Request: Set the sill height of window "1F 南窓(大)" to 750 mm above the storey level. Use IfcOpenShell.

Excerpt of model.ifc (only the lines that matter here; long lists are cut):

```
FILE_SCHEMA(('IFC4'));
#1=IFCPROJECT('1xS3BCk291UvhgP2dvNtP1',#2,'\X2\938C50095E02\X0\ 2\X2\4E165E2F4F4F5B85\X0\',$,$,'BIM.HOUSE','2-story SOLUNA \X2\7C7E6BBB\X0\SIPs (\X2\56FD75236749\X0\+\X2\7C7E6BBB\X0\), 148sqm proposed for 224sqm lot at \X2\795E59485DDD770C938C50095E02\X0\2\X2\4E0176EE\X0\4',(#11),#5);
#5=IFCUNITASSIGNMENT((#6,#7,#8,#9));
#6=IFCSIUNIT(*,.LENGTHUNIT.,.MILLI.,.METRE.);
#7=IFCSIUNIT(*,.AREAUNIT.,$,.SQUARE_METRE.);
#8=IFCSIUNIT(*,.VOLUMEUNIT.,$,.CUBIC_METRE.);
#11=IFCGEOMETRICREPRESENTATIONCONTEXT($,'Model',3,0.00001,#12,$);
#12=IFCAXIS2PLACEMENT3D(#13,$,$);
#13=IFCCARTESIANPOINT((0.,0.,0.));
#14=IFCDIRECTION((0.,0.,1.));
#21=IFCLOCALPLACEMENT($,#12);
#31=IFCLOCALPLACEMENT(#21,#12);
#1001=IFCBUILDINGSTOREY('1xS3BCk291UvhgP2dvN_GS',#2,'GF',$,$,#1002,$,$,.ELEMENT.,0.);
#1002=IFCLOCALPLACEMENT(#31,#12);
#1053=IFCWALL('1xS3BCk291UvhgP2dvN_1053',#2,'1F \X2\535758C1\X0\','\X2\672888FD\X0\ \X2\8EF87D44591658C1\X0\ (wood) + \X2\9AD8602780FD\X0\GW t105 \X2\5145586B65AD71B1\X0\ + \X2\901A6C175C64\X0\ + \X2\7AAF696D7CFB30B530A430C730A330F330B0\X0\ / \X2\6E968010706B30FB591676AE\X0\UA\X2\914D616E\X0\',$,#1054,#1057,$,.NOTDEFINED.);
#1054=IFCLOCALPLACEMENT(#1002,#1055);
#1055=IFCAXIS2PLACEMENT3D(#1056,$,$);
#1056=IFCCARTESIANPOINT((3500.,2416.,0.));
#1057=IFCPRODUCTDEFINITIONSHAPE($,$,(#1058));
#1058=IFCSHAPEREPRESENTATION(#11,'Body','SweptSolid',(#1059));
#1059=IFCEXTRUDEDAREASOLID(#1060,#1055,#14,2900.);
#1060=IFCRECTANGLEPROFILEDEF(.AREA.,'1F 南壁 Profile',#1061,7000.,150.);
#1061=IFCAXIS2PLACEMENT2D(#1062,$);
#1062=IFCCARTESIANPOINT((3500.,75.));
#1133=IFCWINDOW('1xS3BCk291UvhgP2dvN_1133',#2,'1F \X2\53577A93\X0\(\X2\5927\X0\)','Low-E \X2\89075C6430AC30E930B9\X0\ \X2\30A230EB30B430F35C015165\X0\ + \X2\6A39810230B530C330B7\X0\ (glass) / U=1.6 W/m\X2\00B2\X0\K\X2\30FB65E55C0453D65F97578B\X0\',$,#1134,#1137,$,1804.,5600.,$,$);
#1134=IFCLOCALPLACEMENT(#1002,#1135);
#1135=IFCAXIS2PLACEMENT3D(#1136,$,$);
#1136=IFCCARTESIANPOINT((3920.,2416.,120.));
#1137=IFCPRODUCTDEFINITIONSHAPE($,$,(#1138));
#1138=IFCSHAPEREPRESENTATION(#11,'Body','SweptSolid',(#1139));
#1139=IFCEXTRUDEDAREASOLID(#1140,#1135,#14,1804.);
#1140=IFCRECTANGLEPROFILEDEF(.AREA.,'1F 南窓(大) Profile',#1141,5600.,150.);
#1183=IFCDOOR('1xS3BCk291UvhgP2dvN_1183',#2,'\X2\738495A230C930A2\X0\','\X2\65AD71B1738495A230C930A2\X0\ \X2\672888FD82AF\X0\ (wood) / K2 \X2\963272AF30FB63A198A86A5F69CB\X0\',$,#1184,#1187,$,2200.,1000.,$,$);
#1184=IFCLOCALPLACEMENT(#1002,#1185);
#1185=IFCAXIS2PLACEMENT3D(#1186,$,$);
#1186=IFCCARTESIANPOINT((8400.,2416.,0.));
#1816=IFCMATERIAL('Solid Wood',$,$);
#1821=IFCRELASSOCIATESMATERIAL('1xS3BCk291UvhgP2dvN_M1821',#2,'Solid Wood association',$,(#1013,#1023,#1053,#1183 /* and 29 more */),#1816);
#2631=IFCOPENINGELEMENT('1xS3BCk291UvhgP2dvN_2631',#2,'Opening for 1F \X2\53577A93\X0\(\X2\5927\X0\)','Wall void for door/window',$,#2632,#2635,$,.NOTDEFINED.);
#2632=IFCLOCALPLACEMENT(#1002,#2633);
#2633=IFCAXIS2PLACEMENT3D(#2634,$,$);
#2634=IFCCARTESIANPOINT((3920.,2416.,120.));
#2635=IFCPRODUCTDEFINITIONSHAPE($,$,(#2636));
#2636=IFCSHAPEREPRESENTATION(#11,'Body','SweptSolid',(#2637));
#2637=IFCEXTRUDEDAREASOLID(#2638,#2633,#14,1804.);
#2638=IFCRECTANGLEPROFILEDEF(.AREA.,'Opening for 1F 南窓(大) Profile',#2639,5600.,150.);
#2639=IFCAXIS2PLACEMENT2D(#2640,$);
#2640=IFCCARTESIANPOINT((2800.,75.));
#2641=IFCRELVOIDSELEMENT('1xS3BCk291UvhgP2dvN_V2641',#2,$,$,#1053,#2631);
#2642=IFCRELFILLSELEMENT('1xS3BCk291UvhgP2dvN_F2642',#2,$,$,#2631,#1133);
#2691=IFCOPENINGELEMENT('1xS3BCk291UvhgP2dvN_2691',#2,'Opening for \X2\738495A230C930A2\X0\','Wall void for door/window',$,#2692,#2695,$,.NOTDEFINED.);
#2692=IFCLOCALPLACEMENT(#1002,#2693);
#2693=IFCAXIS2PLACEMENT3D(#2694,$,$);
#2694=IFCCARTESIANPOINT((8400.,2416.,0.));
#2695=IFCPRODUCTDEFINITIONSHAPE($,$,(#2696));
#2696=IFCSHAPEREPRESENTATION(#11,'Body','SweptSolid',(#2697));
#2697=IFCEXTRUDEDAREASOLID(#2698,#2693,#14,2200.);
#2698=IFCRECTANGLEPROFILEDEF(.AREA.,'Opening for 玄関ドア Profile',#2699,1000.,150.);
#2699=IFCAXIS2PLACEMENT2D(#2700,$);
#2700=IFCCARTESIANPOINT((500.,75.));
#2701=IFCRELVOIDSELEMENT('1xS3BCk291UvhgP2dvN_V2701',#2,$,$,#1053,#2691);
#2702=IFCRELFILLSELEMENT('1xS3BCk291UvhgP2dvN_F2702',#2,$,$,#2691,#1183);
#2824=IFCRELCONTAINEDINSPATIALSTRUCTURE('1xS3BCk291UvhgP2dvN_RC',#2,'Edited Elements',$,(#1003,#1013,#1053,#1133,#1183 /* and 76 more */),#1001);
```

```python
import numpy as np
import ifcopenshell
import ifcopenshell.api.geometry
import ifcopenshell.geom
import ifcopenshell.util.element
import ifcopenshell.util.placement
import ifcopenshell.util.shape
import ifcopenshell.util.unit

model = ifcopenshell.open("model.ifc")
unit_scale = ifcopenshell.util.unit.calculate_unit_scale(model)

window = model.by_guid("1xS3BCk291UvhgP2dvN_1133")
opening = window.FillsVoids[0].RelatingOpeningElement
storey = ifcopenshell.util.element.get_container(window, ifc_class="IfcBuildingStorey")
level = ifcopenshell.util.placement.get_local_placement(storey.ObjectPlacement)[2, 3]

# The opening's origin need not be at the sill, so measure its lowest point.
shape = ifcopenshell.geom.create_shape(ifcopenshell.geom.settings(), opening)
bottom = ifcopenshell.util.shape.get_shape_bottom_elevation(shape, shape.geometry) / unit_scale
dz = level + 0.75 / unit_scale - bottom

shift = np.array([0.0, 0.0, dz])
# The window is not placed relative to its opening, so move both.
for product in (opening, window):
    matrix = ifcopenshell.util.placement.get_local_placement(product.ObjectPlacement)
    matrix[:3, 3] += shift
    ifcopenshell.api.geometry.edit_object_placement(model, product=product, matrix=matrix, is_si=False)

print(f"moved by {dz * unit_scale:+.3f} m")

model.write("model_rev.ifc")
```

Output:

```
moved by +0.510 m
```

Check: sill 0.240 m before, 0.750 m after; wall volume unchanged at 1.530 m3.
